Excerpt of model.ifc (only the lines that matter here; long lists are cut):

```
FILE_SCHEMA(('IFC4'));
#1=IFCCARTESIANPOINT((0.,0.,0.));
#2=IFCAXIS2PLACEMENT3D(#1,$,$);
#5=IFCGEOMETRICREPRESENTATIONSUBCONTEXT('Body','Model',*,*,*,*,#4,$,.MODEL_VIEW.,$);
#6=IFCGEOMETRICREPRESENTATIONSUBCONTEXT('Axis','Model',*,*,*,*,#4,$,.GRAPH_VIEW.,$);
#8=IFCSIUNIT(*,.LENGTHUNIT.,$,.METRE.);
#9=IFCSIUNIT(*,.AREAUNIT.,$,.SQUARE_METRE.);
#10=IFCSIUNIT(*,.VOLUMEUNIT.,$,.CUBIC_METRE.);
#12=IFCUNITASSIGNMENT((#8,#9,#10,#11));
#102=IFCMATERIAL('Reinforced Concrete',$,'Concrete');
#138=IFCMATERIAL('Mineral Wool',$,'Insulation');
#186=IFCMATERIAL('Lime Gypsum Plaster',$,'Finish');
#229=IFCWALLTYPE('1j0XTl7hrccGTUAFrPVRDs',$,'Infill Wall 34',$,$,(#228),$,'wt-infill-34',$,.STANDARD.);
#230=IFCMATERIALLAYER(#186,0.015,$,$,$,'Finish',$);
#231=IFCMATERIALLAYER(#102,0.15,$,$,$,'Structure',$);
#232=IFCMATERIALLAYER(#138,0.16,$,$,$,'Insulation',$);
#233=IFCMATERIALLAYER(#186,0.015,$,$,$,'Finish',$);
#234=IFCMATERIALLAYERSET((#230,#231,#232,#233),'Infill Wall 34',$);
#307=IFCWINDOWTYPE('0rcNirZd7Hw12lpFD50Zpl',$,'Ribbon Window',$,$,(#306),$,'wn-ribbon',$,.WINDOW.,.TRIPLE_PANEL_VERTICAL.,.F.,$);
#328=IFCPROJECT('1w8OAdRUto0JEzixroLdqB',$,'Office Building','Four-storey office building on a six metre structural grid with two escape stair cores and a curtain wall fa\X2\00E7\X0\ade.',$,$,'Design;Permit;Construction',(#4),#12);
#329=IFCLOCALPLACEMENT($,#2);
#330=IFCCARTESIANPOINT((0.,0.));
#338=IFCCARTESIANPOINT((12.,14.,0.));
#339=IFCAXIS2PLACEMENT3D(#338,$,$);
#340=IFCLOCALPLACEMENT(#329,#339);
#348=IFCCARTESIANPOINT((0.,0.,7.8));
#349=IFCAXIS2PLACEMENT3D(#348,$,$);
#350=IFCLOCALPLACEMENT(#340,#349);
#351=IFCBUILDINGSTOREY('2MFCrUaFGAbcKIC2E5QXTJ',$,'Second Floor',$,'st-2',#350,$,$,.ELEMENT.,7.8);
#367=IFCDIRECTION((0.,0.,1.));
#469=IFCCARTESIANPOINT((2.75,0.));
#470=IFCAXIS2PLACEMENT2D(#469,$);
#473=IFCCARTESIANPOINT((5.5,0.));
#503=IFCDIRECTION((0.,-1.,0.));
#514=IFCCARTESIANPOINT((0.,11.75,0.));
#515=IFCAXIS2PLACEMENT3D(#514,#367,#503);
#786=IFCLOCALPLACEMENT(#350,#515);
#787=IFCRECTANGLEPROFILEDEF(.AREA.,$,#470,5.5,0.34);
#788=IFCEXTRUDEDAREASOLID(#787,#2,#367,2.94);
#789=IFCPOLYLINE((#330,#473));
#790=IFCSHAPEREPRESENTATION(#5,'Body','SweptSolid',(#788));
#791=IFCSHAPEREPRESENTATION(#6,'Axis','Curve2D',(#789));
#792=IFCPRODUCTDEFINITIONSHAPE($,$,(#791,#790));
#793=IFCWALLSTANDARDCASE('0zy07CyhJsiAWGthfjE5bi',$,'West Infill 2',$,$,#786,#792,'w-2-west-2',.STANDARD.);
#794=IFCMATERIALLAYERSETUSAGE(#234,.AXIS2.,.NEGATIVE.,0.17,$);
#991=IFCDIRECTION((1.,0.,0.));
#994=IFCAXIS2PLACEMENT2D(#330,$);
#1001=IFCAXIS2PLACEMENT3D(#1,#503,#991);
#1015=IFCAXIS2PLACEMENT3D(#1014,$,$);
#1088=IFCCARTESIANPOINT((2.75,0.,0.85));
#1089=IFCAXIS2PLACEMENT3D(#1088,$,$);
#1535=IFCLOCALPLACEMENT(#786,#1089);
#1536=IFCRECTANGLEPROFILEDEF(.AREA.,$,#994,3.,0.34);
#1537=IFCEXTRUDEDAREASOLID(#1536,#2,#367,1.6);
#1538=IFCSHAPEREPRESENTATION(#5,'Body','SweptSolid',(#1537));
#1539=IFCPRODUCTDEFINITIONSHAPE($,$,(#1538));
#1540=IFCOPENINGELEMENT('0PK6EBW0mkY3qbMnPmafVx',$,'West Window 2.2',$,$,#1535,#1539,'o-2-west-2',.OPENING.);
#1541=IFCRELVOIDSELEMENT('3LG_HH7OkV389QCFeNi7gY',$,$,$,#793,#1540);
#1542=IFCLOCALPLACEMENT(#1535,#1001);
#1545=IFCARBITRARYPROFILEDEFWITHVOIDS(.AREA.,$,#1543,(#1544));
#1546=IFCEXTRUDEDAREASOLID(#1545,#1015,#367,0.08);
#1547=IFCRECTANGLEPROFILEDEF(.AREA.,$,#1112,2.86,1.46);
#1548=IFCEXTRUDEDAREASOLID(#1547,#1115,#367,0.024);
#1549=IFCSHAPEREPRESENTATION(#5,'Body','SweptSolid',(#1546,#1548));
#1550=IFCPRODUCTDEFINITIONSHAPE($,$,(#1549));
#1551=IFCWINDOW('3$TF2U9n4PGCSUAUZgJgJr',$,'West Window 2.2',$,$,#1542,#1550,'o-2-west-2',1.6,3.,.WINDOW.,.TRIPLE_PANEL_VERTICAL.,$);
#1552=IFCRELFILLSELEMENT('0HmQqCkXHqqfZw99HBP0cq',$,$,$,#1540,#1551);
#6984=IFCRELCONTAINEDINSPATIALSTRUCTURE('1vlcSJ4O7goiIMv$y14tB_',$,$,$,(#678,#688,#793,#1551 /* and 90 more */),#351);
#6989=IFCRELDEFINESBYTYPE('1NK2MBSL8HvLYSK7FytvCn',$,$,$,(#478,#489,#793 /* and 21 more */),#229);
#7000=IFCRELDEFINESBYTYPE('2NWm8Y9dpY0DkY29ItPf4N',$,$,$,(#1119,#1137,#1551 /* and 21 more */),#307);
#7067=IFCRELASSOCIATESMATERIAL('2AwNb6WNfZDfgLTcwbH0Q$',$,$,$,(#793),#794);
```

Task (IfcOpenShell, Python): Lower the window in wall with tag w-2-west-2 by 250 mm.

```python
import numpy as np
import ifcopenshell
import ifcopenshell.api.geometry
import ifcopenshell.util.placement
import ifcopenshell.util.unit

model = ifcopenshell.open("model.ifc")
unit_scale = ifcopenshell.util.unit.calculate_unit_scale(model)

window = model.by_guid("3$TF2U9n4PGCSUAUZgJgJr")
opening = window.FillsVoids[0].RelatingOpeningElement
dz = -0.25 / unit_scale

shift = np.array([0.0, 0.0, dz])
# The window is placed relative to its opening, so it follows when the opening moves.
matrix = ifcopenshell.util.placement.get_local_placement(opening.ObjectPlacement)
matrix[:3, 3] += shift
ifcopenshell.api.geometry.edit_object_placement(
    model, product=opening, matrix=matrix, is_si=False, should_transform_children=True
)

print(f"moved by {dz * unit_scale:+.3f} m")

model.write("model_v2.ifc")
```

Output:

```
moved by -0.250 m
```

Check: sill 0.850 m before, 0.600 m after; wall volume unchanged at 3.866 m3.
